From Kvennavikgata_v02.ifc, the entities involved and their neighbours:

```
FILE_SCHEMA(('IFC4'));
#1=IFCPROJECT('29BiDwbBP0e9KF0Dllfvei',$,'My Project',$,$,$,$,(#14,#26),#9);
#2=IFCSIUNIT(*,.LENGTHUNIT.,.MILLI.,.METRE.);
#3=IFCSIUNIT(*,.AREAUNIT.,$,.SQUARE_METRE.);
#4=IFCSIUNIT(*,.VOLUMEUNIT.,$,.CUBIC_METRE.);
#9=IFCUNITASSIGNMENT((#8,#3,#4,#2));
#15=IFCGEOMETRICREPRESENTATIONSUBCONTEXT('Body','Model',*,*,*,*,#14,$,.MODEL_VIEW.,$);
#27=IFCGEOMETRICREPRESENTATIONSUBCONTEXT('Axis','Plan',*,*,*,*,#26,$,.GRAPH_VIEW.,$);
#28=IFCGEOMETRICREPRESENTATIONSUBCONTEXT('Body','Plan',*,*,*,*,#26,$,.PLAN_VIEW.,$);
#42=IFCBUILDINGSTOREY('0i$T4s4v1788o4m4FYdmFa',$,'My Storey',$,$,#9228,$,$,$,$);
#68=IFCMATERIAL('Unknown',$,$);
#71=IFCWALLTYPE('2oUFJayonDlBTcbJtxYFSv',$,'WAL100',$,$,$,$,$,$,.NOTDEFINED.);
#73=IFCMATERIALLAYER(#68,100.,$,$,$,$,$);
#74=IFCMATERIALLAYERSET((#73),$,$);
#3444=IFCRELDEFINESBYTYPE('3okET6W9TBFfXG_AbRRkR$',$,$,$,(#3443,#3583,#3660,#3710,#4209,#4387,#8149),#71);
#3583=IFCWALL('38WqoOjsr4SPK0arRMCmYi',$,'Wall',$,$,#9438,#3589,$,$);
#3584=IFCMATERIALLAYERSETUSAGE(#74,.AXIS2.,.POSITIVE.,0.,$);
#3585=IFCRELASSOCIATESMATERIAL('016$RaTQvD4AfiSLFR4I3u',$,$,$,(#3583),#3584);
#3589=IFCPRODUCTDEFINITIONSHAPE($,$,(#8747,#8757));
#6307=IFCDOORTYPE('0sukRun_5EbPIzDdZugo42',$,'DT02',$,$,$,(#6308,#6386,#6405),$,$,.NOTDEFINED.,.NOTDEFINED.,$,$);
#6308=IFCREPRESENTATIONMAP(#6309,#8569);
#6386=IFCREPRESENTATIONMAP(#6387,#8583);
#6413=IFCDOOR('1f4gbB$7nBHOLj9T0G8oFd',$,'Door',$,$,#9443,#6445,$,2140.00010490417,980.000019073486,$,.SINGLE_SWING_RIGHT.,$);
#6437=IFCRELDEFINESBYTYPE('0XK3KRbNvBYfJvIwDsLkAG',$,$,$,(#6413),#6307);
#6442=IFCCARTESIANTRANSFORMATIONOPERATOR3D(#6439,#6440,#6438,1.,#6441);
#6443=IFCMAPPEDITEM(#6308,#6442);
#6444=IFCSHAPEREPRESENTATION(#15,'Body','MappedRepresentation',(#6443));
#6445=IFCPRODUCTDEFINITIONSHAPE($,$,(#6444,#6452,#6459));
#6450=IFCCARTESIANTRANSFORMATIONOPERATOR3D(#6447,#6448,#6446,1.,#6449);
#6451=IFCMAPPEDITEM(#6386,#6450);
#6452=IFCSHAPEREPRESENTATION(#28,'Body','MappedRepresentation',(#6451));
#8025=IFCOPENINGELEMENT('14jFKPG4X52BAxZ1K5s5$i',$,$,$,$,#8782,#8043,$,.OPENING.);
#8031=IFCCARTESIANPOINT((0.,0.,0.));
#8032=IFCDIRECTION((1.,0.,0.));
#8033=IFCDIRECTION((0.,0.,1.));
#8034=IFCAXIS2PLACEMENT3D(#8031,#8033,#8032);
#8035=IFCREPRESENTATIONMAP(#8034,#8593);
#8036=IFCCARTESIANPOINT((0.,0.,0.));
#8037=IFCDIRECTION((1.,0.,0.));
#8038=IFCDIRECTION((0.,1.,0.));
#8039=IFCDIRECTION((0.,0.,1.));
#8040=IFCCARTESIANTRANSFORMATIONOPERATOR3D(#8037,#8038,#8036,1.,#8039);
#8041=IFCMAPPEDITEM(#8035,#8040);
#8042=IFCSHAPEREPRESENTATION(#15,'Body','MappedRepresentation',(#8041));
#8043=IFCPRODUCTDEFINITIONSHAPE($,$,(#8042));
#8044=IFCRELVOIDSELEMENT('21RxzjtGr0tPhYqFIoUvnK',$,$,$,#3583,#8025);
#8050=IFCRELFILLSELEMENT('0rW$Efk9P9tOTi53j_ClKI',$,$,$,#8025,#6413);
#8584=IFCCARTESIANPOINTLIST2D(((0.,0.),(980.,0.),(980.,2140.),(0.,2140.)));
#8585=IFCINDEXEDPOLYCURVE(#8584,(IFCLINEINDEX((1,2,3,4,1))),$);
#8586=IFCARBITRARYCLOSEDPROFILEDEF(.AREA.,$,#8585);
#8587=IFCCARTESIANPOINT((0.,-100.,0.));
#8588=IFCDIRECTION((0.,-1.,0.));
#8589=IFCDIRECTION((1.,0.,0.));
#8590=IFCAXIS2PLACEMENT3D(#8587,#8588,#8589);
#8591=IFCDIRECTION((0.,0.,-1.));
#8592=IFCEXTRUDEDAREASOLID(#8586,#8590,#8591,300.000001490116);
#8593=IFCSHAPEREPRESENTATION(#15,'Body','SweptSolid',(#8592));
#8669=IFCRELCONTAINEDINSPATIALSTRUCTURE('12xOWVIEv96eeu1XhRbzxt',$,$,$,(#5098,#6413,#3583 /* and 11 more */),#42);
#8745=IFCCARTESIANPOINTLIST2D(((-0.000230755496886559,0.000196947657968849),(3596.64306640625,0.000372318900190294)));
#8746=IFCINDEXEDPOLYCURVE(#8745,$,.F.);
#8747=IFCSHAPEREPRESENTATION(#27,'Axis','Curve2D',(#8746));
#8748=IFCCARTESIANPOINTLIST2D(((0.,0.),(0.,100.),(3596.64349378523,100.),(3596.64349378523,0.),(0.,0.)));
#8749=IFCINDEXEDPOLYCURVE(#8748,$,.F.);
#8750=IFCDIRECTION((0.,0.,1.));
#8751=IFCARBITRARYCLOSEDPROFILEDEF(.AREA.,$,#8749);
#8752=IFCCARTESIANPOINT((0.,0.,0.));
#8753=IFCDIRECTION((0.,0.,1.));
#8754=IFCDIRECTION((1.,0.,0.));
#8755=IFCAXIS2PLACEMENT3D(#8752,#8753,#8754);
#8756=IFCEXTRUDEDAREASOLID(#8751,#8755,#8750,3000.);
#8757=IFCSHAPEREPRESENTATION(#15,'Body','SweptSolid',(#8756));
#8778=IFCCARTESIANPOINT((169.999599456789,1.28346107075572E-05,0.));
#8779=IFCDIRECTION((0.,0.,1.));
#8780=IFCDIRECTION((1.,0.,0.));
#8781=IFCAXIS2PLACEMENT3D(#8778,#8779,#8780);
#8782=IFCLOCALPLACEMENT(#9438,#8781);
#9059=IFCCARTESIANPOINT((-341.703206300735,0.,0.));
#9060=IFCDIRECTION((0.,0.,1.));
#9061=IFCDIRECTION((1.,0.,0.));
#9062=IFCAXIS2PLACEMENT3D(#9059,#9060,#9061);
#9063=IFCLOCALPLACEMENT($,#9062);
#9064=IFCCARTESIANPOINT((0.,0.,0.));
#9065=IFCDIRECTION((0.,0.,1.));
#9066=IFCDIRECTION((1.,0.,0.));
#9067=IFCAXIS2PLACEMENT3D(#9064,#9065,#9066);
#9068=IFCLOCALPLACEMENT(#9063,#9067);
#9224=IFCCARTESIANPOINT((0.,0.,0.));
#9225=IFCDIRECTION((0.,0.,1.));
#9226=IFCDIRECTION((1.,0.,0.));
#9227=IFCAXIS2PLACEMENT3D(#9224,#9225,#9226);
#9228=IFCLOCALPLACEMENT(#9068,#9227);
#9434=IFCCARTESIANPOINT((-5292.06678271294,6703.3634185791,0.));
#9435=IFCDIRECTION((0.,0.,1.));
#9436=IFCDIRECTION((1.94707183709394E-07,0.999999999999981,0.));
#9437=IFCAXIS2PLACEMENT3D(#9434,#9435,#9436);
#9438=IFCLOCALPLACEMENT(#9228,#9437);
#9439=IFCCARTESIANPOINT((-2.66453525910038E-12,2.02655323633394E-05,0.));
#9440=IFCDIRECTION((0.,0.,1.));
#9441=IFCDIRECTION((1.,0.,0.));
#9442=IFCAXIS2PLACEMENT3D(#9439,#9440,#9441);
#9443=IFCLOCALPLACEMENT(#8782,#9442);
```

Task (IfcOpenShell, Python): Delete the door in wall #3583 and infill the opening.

```python
import ifcopenshell
import ifcopenshell.api.feature
import ifcopenshell.api.root
import ifcopenshell.geom
import ifcopenshell.util.shape

model = ifcopenshell.open("Kvennavikgata_v02.ifc")
settings = ifcopenshell.geom.settings()


def volume(element):
    """Net volume in cubic metres, openings subtracted."""
    shape = ifcopenshell.geom.create_shape(settings, element)
    return ifcopenshell.util.shape.get_volume(shape.geometry)


door = model.by_guid("1f4gbB$7nBHOLj9T0G8oFd")
opening = door.FillsVoids[0].RelatingOpeningElement
wall = opening.VoidsElements[0].RelatingBuildingElement
before = volume(wall)

ifcopenshell.api.root.remove_product(model, product=door)
ifcopenshell.api.feature.remove_feature(model, feature=opening)

after = volume(wall)

print(f"wall volume {before:.3f} -> {after:.3f} m3")

model.write("Kvennavikgata_v02_rev.ifc")
```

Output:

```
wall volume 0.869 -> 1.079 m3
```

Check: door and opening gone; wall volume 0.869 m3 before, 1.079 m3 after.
